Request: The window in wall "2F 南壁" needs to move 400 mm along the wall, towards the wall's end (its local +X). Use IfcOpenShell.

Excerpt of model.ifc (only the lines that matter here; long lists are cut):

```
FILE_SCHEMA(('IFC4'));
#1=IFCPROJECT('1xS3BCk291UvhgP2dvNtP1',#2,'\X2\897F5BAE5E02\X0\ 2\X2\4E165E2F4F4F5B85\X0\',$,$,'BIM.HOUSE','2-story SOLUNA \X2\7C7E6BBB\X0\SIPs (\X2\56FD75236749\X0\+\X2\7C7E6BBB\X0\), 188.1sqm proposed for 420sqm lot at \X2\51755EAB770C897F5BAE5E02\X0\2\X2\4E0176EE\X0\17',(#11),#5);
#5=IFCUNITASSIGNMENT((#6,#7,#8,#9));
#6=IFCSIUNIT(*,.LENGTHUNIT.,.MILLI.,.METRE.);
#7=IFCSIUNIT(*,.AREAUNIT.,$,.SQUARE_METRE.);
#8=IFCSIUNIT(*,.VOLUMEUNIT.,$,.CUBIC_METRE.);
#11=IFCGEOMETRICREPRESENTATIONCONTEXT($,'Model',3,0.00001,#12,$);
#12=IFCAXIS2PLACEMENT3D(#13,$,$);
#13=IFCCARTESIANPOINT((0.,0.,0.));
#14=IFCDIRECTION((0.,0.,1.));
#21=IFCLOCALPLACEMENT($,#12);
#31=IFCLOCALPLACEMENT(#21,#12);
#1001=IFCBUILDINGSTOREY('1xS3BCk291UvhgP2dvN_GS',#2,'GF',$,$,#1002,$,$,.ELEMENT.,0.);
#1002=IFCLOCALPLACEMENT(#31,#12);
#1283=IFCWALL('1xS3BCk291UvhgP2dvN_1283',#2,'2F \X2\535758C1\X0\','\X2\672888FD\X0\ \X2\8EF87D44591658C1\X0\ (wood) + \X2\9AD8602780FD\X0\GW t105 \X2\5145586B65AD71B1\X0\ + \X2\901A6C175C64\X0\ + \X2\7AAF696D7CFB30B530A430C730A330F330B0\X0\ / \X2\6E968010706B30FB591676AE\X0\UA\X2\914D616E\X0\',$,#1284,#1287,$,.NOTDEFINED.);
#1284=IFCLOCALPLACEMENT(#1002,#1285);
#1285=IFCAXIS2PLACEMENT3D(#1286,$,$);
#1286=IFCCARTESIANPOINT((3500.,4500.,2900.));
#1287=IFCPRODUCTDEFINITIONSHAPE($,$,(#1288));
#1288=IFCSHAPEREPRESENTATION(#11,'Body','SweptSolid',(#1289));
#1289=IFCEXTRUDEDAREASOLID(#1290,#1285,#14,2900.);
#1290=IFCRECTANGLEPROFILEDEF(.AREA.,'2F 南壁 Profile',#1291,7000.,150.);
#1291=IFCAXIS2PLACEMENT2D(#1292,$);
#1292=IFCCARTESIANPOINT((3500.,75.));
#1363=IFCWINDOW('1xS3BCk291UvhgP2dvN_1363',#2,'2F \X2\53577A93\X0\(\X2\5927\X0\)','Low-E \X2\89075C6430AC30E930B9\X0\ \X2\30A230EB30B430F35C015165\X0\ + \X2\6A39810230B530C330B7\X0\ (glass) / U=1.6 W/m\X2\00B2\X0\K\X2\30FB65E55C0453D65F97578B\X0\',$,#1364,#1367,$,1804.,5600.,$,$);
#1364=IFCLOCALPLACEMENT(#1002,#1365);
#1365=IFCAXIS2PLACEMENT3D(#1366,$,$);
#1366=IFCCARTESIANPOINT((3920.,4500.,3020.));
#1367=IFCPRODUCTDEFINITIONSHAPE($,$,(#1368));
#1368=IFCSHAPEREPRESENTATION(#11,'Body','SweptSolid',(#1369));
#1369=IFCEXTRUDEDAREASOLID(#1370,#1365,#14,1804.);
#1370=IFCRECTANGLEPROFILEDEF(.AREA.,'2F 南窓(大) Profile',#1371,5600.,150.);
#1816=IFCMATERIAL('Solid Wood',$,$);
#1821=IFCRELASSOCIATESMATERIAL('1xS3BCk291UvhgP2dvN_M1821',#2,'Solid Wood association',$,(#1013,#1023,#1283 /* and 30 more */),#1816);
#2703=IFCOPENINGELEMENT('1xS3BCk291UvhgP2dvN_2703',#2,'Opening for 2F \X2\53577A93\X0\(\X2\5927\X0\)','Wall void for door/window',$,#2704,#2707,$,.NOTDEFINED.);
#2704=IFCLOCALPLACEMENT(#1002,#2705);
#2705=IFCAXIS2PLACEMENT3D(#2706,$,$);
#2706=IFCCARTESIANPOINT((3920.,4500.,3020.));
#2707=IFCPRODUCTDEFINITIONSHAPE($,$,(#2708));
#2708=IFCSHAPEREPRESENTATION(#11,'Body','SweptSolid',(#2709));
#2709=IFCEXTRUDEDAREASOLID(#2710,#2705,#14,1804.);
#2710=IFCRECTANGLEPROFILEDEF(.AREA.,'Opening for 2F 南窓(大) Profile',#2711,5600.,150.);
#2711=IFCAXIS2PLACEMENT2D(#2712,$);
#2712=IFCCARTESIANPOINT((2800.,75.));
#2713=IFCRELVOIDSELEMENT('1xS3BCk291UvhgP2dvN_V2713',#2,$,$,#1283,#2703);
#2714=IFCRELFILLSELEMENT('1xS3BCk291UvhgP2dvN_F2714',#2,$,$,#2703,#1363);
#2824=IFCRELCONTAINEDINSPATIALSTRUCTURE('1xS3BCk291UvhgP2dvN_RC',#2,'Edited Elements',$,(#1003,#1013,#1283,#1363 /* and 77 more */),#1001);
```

```python
import ifcopenshell
import ifcopenshell.api.geometry
import ifcopenshell.util.placement
import ifcopenshell.util.unit

model = ifcopenshell.open("model.ifc")
unit_scale = ifcopenshell.util.unit.calculate_unit_scale(model)

window = model.by_guid("1xS3BCk291UvhgP2dvN_1363")
opening = window.FillsVoids[0].RelatingOpeningElement
wall = opening.VoidsElements[0].RelatingBuildingElement

wall_matrix = ifcopenshell.util.placement.get_local_placement(wall.ObjectPlacement)
shift = wall_matrix[:3, 0] * 0.4 / unit_scale
before = ifcopenshell.util.placement.get_local_placement(window.ObjectPlacement)[:3, 3].copy()

# The window is not placed relative to its opening, so move both.
for product in (opening, window):
    matrix = ifcopenshell.util.placement.get_local_placement(product.ObjectPlacement)
    matrix[:3, 3] += shift
    ifcopenshell.api.geometry.edit_object_placement(model, product=product, matrix=matrix, is_si=False)

after = ifcopenshell.util.placement.get_local_placement(window.ObjectPlacement)[:3, 3]
print("window moved by", (after - before).round(3) + 0.0)

model.write("model_v2.ifc")
```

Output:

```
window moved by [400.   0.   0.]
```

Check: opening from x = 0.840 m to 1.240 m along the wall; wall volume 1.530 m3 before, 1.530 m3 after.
